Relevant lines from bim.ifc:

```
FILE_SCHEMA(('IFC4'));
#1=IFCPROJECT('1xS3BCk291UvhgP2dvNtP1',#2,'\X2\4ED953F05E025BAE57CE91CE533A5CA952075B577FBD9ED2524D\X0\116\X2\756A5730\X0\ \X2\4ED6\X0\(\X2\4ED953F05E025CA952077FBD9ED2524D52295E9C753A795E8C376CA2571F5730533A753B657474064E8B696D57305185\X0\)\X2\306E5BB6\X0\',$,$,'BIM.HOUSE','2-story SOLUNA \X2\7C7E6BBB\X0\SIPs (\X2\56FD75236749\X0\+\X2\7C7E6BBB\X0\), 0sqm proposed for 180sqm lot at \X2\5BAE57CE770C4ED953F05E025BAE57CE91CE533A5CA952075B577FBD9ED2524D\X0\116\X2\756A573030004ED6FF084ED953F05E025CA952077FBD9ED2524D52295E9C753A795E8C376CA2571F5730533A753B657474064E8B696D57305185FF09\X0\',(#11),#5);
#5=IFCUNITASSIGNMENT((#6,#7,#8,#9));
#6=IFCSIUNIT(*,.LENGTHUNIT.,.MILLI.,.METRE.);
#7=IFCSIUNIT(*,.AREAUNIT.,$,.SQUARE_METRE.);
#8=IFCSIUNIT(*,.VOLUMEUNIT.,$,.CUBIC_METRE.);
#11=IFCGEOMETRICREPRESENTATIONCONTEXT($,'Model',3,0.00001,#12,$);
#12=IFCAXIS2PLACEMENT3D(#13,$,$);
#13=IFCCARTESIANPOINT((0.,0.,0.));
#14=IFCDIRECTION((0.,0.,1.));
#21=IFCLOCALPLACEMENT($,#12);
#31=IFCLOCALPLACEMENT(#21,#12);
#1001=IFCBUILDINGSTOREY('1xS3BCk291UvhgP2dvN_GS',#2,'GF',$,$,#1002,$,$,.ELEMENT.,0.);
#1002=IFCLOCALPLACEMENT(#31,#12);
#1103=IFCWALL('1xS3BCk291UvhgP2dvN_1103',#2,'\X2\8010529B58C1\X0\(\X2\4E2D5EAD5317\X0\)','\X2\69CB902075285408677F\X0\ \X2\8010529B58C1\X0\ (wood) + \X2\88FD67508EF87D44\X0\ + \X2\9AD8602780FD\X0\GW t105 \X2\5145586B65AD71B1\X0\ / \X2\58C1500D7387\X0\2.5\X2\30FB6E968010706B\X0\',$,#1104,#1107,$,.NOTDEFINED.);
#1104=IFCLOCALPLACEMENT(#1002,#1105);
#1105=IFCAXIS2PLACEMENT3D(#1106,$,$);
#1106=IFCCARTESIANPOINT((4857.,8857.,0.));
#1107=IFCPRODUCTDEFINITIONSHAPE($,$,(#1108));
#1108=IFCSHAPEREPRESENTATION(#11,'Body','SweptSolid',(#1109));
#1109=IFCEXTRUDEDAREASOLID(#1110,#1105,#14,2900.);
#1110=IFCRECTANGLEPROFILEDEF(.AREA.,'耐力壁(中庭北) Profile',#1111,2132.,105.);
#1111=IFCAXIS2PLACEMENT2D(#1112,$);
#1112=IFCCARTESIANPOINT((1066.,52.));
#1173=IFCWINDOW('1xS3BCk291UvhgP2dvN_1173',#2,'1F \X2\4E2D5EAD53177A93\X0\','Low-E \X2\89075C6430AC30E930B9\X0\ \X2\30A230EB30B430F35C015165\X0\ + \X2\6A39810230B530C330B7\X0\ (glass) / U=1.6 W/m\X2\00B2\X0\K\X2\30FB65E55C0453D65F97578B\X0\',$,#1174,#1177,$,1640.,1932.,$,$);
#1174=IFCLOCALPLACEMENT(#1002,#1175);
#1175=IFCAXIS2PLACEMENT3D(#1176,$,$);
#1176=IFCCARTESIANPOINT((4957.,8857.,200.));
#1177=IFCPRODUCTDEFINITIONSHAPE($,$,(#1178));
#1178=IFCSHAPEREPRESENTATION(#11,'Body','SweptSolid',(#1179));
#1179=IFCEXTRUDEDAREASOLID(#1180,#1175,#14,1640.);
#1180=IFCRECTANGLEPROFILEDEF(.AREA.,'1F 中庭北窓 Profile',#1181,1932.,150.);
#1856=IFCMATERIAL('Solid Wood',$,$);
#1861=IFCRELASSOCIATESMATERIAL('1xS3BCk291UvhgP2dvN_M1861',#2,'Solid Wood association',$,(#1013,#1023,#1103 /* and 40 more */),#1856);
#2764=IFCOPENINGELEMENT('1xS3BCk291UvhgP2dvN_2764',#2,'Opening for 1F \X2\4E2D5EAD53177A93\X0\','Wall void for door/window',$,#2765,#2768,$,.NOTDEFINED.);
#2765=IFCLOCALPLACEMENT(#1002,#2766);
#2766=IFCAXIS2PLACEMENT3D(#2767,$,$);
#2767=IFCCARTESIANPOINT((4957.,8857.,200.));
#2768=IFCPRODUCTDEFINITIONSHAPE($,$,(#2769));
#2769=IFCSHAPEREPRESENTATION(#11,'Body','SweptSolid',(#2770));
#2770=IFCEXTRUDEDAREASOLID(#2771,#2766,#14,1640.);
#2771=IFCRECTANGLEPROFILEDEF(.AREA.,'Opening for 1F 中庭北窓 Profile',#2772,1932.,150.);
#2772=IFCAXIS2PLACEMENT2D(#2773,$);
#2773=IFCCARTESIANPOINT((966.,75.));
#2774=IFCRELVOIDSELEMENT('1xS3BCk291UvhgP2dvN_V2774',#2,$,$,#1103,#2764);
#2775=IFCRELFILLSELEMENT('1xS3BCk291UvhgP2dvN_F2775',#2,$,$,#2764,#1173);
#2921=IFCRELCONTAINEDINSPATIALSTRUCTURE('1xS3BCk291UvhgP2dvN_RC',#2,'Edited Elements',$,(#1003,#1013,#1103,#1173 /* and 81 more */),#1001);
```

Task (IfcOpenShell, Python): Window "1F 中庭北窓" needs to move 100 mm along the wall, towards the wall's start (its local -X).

```python
import ifcopenshell
import ifcopenshell.api.geometry
import ifcopenshell.util.placement

model = ifcopenshell.open("bim.ifc")

window = model.by_guid("1xS3BCk291UvhgP2dvN_1173")
opening = window.FillsVoids[0].RelatingOpeningElement
wall = opening.VoidsElements[0].RelatingBuildingElement

wall_matrix = ifcopenshell.util.placement.get_local_placement(wall.ObjectPlacement)
shift = wall_matrix[:3, 0] * -100.0
before = ifcopenshell.util.placement.get_local_placement(window.ObjectPlacement)[:3, 3].copy()

# The window is not placed relative to its opening, so move both.
for product in (opening, window):
    matrix = ifcopenshell.util.placement.get_local_placement(product.ObjectPlacement)
    matrix[:3, 3] += shift
    ifcopenshell.api.geometry.edit_object_placement(model, product=product, matrix=matrix, is_si=False)

after = ifcopenshell.util.placement.get_local_placement(window.ObjectPlacement)[:3, 3]
print("window moved by", (after - before).round(3) + 0.0)

model.write("bim_edited.ifc")
```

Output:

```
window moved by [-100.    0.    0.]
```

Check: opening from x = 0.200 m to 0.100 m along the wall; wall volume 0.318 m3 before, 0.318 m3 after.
